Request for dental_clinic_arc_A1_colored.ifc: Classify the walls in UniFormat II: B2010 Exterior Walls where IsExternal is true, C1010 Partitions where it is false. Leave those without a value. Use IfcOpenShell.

First a look at what the model holds.

```python
import ifcopenshell
import ifcopenshell.util.element

model = ifcopenshell.open("dental_clinic_arc_A1_colored.ifc")
print(model.schema)
print("classifications:", [c.Name for c in model.by_type("IfcClassification")])
values = [ifcopenshell.util.element.get_pset(e, "Pset_WallCommon", "IsExternal") for e in model.by_type("IfcWall")]
for value in (True, False, None):
    print("IsExternal", value, values.count(value))
```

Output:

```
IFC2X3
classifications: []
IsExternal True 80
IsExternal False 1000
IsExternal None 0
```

```python
import ifcopenshell
import ifcopenshell.api.classification
import ifcopenshell.util.element

model = ifcopenshell.open("dental_clinic_arc_A1_colored.ifc")

# IFC2X3 requires Source and Edition and has no link from the project to the system.
system = model.create_entity("IfcClassification", Source="ASTM", Edition="E1557", Name="UniFormat II")

walls = model.by_type("IfcWall")
external = {e: ifcopenshell.util.element.get_pset(e, "Pset_WallCommon", "IsExternal") for e in walls}
for flag, code, name in ((True, "B2010", "Exterior Walls"), (False, "C1010", "Partitions")):
    products = [e for e in walls if external[e] is flag]
    ifcopenshell.api.classification.add_reference(
        model, products=products, classification=system, identification=code, name=name
    )
    print(code, len(products))

model.write("dental_clinic_arc_A1_colored_rev.ifc")
```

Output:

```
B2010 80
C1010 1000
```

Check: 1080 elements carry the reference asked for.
